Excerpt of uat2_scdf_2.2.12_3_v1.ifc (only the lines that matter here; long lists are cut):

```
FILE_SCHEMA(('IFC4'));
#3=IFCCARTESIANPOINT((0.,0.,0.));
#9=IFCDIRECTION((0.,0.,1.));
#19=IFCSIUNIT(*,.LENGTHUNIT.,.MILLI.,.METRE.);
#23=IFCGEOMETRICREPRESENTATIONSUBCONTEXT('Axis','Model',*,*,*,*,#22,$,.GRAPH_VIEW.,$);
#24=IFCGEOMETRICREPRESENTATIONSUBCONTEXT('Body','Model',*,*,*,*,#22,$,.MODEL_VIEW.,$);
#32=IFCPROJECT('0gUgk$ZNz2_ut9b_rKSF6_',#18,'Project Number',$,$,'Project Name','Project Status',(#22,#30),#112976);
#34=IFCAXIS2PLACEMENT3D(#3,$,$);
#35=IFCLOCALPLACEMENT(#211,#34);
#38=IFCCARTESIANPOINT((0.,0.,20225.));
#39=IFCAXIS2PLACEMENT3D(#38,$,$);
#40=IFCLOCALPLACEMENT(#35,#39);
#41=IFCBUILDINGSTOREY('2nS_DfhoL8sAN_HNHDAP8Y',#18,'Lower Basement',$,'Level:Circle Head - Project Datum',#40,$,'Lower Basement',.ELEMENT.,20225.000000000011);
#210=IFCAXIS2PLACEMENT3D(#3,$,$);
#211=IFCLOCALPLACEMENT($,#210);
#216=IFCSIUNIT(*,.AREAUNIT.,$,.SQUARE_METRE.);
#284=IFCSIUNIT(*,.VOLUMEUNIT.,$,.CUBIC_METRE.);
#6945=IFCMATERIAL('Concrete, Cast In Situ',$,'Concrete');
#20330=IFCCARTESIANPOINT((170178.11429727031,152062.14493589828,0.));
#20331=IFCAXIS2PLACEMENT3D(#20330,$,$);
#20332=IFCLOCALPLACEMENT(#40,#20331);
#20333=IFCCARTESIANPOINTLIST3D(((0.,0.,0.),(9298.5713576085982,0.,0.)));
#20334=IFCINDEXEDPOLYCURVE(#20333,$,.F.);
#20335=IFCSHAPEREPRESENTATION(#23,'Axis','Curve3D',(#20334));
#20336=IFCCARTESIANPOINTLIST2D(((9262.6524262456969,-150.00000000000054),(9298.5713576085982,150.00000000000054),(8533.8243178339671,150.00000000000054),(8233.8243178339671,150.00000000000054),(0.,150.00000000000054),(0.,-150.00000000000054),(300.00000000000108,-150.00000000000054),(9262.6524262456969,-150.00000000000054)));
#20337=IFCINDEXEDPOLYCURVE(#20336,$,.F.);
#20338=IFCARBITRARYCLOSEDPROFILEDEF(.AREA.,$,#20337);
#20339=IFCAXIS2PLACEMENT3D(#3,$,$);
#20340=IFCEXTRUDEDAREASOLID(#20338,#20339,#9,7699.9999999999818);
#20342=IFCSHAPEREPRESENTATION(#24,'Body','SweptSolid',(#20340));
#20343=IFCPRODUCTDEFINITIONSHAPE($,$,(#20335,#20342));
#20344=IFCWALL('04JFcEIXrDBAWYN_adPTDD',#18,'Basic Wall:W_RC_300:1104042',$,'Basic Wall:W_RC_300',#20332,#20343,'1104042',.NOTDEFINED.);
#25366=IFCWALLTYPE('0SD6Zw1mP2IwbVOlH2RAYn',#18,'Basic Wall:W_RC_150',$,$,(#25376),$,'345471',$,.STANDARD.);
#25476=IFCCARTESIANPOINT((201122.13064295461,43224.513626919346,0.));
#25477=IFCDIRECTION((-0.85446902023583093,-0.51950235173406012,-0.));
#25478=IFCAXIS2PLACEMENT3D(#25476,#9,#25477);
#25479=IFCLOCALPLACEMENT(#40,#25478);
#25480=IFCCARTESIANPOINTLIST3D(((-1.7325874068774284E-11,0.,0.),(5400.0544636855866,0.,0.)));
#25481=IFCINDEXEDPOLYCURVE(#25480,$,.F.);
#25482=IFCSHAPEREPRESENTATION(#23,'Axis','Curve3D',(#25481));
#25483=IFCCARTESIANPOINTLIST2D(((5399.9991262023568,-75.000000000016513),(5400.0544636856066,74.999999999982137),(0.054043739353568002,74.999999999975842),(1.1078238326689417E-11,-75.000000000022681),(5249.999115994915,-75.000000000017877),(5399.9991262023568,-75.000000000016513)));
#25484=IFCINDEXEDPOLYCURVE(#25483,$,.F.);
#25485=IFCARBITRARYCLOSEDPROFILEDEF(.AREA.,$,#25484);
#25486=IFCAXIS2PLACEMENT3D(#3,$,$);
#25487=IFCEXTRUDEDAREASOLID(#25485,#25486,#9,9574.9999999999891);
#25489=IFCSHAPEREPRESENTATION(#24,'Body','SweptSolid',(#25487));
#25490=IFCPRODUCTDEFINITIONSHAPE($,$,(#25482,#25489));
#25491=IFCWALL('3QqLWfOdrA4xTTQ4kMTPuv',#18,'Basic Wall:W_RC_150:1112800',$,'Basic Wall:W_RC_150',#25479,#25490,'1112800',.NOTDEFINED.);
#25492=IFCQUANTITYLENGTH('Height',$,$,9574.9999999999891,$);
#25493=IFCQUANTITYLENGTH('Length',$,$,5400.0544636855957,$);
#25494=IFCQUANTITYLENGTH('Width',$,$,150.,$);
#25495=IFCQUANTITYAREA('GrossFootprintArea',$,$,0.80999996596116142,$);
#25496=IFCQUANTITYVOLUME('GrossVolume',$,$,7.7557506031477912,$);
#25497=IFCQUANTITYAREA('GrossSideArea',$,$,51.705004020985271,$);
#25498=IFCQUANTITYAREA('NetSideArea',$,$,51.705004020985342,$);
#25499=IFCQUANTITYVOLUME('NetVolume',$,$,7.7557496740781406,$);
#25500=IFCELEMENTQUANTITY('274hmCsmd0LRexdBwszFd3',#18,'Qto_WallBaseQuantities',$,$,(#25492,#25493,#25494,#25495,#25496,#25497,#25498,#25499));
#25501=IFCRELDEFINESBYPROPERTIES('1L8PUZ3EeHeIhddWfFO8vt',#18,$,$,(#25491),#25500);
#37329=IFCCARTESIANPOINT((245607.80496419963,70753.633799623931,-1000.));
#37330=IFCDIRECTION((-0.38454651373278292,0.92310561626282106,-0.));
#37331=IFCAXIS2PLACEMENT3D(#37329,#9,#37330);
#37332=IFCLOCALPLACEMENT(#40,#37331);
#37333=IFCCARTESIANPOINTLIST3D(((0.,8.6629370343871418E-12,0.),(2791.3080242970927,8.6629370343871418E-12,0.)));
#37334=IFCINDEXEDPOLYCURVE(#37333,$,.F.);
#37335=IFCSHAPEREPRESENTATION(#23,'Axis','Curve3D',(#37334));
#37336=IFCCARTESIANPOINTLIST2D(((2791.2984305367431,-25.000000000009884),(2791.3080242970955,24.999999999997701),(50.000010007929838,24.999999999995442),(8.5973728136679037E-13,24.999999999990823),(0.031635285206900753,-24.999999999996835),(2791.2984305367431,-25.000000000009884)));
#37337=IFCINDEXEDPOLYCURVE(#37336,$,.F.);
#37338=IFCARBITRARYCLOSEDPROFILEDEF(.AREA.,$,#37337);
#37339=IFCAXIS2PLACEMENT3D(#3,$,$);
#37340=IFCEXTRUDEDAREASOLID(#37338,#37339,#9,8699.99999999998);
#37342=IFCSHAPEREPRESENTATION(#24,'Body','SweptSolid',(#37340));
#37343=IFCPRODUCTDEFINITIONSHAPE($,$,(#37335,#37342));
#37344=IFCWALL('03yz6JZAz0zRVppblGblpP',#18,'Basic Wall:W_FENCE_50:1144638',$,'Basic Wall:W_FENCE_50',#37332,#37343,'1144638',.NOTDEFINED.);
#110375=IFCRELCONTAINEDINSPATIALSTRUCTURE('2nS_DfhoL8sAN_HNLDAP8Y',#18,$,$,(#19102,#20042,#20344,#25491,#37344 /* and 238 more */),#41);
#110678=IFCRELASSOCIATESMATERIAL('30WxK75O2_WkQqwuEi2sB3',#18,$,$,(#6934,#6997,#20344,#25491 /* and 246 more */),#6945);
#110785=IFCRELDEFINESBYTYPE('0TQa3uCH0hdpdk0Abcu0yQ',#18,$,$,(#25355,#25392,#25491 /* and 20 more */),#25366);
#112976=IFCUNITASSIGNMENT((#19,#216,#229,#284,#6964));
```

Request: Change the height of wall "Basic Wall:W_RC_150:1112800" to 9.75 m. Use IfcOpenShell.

```python
import ifcopenshell
import ifcopenshell.api.pset
import ifcopenshell.geom
import ifcopenshell.util.element
import ifcopenshell.util.representation
import ifcopenshell.util.shape
import ifcopenshell.util.unit

model = ifcopenshell.open("uat2_scdf_2.2.12_3_v1.ifc")
unit_scale = ifcopenshell.util.unit.calculate_unit_scale(model)
area_scale = ifcopenshell.util.unit.calculate_unit_scale(model, "AREAUNIT")
volume_scale = ifcopenshell.util.unit.calculate_unit_scale(model, "VOLUMEUNIT")
settings = ifcopenshell.geom.settings()


def volume(element):
    """Net volume in cubic metres, openings subtracted."""
    shape = ifcopenshell.geom.create_shape(settings, element)
    return ifcopenshell.util.shape.get_volume(shape.geometry)


wall = model.by_id(25491)
before = volume(wall)

body = ifcopenshell.util.representation.get_representation(wall, "Model", "Body")
solid = body.Items[0]
old_height = solid.Depth
solid.Depth = 9750.0
after = volume(wall)
thickness = 0.15  # wall thickness in metres

# Update the stored height, areas and volumes.
qto = model.by_id(ifcopenshell.util.element.get_pset(wall, "Qto_WallBaseQuantities", should_inherit=False)["id"])
ifcopenshell.api.pset.edit_qto(model, qto=qto, properties={
    "Height": solid.Depth,
    "GrossVolume": ifcopenshell.util.element.get_pset(wall, "Qto_WallBaseQuantities", "GrossVolume") * solid.Depth / old_height,
    "GrossSideArea": ifcopenshell.util.element.get_pset(wall, "Qto_WallBaseQuantities", "GrossSideArea") * solid.Depth / old_height,
    "NetSideArea": after / thickness / area_scale,
    "NetVolume": after / volume_scale,
})

print(f"height {old_height:g} -> {solid.Depth:g}, volume {before:.3f} -> {after:.3f} m3")

model.write("uat2_scdf_2.2.12_3_v1_updated.ifc")
```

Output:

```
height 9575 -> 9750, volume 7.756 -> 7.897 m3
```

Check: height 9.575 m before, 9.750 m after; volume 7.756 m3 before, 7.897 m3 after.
